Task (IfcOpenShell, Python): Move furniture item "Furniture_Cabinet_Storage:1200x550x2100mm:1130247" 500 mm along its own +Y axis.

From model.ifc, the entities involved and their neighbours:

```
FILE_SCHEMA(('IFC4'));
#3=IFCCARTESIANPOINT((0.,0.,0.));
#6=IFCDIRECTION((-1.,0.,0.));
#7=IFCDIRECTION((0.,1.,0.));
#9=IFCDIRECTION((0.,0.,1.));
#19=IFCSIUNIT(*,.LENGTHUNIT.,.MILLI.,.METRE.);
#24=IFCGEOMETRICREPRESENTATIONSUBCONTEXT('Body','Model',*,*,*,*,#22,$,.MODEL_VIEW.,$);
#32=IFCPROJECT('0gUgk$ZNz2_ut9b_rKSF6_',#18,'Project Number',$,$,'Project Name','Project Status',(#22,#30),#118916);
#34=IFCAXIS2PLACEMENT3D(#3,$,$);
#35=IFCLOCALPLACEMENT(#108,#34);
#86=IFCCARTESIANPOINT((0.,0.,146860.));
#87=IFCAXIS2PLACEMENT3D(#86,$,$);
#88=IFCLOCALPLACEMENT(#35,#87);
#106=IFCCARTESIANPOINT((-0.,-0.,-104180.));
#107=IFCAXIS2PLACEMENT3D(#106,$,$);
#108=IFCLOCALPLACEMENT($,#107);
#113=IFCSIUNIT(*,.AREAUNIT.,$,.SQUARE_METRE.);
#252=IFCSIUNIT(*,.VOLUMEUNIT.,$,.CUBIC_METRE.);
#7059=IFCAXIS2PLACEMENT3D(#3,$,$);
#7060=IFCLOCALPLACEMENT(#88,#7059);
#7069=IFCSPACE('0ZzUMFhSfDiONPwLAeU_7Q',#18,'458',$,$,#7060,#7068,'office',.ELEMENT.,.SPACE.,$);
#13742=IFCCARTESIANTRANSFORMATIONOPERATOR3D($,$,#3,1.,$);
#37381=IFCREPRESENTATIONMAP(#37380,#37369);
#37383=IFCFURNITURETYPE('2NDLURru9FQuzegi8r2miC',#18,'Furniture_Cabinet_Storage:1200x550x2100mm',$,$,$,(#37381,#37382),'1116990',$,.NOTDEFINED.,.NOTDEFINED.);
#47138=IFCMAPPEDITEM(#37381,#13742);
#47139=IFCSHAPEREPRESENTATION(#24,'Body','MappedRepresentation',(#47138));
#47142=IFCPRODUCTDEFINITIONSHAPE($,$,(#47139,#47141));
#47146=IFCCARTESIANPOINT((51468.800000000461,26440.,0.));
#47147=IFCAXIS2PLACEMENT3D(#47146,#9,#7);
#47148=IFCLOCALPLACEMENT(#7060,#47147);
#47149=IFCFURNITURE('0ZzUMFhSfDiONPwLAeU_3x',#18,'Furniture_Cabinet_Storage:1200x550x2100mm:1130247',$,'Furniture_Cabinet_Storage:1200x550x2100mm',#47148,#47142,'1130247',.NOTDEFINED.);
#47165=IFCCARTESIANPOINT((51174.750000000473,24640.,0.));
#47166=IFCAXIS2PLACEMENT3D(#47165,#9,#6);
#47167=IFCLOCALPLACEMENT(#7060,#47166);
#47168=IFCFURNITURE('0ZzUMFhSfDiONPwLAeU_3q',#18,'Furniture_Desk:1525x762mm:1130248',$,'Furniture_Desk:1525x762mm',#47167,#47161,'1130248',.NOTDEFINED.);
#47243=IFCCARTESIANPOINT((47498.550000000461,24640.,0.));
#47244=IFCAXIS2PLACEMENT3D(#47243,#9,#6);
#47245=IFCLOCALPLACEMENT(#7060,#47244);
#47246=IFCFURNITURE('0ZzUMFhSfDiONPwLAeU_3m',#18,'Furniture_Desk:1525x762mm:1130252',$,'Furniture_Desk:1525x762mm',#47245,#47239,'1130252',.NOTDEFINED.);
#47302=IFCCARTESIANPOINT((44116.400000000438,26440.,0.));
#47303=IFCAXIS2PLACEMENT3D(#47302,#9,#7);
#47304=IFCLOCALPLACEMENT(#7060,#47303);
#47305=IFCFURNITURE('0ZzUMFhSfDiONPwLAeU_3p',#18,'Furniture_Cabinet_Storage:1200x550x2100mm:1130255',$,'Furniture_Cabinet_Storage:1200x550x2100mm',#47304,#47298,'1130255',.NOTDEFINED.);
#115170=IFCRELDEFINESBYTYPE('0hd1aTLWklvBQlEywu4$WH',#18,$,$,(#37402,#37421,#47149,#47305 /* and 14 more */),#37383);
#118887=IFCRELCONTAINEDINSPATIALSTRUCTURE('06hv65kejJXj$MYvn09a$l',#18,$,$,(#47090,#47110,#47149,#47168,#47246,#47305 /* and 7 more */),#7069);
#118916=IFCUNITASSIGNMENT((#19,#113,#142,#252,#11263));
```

```python
import ifcopenshell
import ifcopenshell.api.geometry
import ifcopenshell.util.placement
import ifcopenshell.util.unit

model = ifcopenshell.open("model.ifc")
unit_scale = ifcopenshell.util.unit.calculate_unit_scale(model)

item = model.by_guid("0ZzUMFhSfDiONPwLAeU_3x")
matrix = ifcopenshell.util.placement.get_local_placement(item.ObjectPlacement)
matrix[:3, 3] += matrix[:3, 1] * 0.5 / unit_scale
ifcopenshell.api.geometry.edit_object_placement(model, product=item, matrix=matrix, is_si=False)

print(ifcopenshell.util.placement.get_local_placement(item.ObjectPlacement).round(3) + 0.0)

model.write("model_v2.ifc")
```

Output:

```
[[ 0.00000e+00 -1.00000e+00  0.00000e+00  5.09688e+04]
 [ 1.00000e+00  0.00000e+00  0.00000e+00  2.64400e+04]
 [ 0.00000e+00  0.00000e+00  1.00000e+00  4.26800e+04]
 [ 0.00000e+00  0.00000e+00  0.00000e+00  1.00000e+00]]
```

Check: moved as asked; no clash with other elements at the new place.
